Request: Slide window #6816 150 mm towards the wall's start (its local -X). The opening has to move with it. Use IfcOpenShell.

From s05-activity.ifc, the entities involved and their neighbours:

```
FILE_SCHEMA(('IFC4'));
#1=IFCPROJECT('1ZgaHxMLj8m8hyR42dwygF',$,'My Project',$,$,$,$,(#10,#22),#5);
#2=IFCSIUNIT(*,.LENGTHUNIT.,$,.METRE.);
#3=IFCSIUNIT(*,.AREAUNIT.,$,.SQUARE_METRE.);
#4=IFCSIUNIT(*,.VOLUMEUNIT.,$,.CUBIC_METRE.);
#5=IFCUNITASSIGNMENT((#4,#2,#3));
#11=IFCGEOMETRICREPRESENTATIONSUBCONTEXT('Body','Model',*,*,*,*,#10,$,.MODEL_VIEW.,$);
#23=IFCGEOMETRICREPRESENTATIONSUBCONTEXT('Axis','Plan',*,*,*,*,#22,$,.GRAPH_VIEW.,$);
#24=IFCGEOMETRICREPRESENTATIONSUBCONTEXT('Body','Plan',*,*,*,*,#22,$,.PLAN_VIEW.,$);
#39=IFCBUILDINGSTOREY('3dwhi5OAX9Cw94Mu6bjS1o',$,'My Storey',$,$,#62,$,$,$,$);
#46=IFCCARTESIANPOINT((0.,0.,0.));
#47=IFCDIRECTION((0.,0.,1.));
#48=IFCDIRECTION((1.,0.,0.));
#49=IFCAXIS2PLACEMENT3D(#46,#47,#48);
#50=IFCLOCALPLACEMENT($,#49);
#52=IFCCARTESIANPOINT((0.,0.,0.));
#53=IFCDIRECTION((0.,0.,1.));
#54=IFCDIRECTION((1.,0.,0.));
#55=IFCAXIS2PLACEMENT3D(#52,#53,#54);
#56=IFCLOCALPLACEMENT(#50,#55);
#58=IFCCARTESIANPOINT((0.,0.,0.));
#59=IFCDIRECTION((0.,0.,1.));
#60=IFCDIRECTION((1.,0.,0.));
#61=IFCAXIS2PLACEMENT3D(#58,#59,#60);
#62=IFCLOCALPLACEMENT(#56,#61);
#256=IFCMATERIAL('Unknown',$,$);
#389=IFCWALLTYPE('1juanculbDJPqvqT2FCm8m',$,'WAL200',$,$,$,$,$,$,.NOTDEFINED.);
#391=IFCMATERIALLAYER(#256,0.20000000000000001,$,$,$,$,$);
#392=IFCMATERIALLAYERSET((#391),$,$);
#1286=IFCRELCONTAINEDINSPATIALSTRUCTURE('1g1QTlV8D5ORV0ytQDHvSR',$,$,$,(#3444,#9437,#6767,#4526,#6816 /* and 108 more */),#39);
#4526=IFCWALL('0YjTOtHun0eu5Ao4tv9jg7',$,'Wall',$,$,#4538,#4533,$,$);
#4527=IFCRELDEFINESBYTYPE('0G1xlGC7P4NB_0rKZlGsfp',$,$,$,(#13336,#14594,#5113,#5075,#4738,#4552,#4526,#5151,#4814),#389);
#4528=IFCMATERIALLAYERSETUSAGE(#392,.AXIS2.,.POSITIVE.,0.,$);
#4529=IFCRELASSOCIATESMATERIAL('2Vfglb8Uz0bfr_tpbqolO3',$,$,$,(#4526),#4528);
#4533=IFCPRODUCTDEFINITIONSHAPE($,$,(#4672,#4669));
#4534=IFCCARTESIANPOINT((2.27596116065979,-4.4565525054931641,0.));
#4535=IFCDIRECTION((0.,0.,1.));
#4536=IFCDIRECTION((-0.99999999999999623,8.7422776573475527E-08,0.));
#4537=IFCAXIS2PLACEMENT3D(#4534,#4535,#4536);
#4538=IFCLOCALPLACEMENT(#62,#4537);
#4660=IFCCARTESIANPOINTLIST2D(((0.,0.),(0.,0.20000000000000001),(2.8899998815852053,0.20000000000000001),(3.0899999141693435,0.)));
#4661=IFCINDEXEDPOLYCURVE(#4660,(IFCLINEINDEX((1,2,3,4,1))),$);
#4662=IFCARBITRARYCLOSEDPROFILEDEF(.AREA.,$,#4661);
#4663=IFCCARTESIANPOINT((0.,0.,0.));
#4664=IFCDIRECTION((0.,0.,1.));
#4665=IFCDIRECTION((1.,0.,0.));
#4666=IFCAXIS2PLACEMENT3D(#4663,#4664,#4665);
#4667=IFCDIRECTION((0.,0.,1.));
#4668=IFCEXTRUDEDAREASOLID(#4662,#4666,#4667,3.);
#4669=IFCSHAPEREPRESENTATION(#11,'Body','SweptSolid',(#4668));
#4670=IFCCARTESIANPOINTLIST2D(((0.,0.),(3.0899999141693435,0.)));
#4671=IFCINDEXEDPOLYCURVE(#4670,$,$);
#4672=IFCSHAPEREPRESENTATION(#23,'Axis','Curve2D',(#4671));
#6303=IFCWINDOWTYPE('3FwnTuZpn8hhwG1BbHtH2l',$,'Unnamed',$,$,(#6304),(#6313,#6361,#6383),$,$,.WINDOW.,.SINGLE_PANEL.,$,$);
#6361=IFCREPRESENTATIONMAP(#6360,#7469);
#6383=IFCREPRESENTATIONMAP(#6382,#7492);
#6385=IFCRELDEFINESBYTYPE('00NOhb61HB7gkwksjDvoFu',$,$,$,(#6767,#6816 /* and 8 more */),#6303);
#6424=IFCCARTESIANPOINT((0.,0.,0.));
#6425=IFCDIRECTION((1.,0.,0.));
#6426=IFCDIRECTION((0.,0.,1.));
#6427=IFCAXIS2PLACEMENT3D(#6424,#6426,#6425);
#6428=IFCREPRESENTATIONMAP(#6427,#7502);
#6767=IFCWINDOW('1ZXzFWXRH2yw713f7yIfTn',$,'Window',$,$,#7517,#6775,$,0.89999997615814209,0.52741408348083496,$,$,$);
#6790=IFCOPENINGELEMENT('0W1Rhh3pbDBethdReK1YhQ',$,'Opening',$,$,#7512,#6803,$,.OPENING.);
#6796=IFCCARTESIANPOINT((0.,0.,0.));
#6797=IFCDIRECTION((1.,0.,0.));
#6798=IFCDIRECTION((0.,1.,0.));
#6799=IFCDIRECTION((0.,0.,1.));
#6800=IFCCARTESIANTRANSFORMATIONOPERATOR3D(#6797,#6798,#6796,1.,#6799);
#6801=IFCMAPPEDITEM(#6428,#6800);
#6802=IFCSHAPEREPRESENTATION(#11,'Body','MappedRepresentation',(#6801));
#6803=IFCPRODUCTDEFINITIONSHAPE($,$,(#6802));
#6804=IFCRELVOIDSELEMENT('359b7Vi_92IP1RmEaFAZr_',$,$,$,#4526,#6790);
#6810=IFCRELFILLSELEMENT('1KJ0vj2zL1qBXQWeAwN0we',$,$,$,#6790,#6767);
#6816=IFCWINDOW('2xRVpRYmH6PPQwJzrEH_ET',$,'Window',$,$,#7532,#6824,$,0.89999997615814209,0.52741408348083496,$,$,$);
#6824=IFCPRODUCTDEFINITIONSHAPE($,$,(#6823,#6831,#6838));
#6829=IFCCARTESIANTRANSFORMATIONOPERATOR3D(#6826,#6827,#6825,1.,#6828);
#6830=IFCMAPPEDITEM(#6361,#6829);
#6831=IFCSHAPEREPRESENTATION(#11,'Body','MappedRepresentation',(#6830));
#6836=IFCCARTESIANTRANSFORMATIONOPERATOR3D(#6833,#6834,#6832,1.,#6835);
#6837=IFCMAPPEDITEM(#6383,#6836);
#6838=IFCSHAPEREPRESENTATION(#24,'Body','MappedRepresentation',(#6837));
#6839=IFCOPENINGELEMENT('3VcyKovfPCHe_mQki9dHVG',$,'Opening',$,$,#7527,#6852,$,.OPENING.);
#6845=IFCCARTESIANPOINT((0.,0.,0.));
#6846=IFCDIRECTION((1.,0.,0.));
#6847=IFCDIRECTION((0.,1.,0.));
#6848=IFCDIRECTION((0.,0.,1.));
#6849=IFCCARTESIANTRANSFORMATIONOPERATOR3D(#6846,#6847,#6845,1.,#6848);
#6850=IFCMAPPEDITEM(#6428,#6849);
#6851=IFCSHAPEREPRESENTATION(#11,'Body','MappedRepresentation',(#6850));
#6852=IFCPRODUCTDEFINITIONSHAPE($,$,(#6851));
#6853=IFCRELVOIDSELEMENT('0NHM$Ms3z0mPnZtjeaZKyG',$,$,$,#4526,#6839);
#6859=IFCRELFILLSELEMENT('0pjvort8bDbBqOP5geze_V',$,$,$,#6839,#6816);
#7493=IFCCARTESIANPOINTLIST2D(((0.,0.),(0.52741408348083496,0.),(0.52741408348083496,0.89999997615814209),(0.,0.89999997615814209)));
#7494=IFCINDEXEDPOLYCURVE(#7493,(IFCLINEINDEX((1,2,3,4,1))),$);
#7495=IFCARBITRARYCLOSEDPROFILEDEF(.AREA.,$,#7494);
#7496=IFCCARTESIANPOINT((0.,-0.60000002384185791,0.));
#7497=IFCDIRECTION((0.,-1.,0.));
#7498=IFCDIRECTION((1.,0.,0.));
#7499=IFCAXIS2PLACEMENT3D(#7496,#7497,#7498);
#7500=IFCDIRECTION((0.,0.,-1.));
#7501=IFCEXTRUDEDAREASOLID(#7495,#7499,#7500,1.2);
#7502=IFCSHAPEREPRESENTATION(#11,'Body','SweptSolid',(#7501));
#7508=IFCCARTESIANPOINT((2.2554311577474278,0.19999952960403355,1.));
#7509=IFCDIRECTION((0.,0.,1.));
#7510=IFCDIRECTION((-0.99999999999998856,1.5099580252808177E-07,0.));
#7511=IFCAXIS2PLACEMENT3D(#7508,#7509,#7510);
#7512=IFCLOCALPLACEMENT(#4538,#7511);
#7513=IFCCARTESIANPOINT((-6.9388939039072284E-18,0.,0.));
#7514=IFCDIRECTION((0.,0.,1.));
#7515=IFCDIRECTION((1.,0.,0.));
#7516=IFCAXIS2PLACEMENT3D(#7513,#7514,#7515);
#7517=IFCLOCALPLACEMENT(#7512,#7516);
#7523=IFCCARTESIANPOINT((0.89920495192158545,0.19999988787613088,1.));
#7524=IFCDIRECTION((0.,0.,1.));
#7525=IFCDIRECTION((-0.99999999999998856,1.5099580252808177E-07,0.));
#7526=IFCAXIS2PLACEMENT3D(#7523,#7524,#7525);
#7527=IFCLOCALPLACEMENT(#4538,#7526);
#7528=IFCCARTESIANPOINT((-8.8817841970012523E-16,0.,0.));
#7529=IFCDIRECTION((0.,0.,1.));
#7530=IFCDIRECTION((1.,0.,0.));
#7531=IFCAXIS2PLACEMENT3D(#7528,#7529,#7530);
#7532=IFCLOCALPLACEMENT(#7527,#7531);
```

```python
import ifcopenshell
import ifcopenshell.api.geometry
import ifcopenshell.util.placement
import ifcopenshell.util.unit

model = ifcopenshell.open("s05-activity.ifc")
unit_scale = ifcopenshell.util.unit.calculate_unit_scale(model)

window = model.by_guid("2xRVpRYmH6PPQwJzrEH_ET")
opening = window.FillsVoids[0].RelatingOpeningElement
wall = opening.VoidsElements[0].RelatingBuildingElement

wall_matrix = ifcopenshell.util.placement.get_local_placement(wall.ObjectPlacement)
shift = wall_matrix[:3, 0] * -0.15 / unit_scale
before = ifcopenshell.util.placement.get_local_placement(window.ObjectPlacement)[:3, 3].copy()

# The window is placed relative to its opening, so it follows when the opening moves.
matrix = ifcopenshell.util.placement.get_local_placement(opening.ObjectPlacement)
matrix[:3, 3] += shift
ifcopenshell.api.geometry.edit_object_placement(
    model, product=opening, matrix=matrix, is_si=False, should_transform_children=True
)

after = ifcopenshell.util.placement.get_local_placement(window.ObjectPlacement)[:3, 3]
print("window moved by", (after - before).round(3) + 0.0)

model.write("s05-activity_v2.ifc")
```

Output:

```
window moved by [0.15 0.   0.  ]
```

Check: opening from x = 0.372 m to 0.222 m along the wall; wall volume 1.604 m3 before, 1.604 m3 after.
